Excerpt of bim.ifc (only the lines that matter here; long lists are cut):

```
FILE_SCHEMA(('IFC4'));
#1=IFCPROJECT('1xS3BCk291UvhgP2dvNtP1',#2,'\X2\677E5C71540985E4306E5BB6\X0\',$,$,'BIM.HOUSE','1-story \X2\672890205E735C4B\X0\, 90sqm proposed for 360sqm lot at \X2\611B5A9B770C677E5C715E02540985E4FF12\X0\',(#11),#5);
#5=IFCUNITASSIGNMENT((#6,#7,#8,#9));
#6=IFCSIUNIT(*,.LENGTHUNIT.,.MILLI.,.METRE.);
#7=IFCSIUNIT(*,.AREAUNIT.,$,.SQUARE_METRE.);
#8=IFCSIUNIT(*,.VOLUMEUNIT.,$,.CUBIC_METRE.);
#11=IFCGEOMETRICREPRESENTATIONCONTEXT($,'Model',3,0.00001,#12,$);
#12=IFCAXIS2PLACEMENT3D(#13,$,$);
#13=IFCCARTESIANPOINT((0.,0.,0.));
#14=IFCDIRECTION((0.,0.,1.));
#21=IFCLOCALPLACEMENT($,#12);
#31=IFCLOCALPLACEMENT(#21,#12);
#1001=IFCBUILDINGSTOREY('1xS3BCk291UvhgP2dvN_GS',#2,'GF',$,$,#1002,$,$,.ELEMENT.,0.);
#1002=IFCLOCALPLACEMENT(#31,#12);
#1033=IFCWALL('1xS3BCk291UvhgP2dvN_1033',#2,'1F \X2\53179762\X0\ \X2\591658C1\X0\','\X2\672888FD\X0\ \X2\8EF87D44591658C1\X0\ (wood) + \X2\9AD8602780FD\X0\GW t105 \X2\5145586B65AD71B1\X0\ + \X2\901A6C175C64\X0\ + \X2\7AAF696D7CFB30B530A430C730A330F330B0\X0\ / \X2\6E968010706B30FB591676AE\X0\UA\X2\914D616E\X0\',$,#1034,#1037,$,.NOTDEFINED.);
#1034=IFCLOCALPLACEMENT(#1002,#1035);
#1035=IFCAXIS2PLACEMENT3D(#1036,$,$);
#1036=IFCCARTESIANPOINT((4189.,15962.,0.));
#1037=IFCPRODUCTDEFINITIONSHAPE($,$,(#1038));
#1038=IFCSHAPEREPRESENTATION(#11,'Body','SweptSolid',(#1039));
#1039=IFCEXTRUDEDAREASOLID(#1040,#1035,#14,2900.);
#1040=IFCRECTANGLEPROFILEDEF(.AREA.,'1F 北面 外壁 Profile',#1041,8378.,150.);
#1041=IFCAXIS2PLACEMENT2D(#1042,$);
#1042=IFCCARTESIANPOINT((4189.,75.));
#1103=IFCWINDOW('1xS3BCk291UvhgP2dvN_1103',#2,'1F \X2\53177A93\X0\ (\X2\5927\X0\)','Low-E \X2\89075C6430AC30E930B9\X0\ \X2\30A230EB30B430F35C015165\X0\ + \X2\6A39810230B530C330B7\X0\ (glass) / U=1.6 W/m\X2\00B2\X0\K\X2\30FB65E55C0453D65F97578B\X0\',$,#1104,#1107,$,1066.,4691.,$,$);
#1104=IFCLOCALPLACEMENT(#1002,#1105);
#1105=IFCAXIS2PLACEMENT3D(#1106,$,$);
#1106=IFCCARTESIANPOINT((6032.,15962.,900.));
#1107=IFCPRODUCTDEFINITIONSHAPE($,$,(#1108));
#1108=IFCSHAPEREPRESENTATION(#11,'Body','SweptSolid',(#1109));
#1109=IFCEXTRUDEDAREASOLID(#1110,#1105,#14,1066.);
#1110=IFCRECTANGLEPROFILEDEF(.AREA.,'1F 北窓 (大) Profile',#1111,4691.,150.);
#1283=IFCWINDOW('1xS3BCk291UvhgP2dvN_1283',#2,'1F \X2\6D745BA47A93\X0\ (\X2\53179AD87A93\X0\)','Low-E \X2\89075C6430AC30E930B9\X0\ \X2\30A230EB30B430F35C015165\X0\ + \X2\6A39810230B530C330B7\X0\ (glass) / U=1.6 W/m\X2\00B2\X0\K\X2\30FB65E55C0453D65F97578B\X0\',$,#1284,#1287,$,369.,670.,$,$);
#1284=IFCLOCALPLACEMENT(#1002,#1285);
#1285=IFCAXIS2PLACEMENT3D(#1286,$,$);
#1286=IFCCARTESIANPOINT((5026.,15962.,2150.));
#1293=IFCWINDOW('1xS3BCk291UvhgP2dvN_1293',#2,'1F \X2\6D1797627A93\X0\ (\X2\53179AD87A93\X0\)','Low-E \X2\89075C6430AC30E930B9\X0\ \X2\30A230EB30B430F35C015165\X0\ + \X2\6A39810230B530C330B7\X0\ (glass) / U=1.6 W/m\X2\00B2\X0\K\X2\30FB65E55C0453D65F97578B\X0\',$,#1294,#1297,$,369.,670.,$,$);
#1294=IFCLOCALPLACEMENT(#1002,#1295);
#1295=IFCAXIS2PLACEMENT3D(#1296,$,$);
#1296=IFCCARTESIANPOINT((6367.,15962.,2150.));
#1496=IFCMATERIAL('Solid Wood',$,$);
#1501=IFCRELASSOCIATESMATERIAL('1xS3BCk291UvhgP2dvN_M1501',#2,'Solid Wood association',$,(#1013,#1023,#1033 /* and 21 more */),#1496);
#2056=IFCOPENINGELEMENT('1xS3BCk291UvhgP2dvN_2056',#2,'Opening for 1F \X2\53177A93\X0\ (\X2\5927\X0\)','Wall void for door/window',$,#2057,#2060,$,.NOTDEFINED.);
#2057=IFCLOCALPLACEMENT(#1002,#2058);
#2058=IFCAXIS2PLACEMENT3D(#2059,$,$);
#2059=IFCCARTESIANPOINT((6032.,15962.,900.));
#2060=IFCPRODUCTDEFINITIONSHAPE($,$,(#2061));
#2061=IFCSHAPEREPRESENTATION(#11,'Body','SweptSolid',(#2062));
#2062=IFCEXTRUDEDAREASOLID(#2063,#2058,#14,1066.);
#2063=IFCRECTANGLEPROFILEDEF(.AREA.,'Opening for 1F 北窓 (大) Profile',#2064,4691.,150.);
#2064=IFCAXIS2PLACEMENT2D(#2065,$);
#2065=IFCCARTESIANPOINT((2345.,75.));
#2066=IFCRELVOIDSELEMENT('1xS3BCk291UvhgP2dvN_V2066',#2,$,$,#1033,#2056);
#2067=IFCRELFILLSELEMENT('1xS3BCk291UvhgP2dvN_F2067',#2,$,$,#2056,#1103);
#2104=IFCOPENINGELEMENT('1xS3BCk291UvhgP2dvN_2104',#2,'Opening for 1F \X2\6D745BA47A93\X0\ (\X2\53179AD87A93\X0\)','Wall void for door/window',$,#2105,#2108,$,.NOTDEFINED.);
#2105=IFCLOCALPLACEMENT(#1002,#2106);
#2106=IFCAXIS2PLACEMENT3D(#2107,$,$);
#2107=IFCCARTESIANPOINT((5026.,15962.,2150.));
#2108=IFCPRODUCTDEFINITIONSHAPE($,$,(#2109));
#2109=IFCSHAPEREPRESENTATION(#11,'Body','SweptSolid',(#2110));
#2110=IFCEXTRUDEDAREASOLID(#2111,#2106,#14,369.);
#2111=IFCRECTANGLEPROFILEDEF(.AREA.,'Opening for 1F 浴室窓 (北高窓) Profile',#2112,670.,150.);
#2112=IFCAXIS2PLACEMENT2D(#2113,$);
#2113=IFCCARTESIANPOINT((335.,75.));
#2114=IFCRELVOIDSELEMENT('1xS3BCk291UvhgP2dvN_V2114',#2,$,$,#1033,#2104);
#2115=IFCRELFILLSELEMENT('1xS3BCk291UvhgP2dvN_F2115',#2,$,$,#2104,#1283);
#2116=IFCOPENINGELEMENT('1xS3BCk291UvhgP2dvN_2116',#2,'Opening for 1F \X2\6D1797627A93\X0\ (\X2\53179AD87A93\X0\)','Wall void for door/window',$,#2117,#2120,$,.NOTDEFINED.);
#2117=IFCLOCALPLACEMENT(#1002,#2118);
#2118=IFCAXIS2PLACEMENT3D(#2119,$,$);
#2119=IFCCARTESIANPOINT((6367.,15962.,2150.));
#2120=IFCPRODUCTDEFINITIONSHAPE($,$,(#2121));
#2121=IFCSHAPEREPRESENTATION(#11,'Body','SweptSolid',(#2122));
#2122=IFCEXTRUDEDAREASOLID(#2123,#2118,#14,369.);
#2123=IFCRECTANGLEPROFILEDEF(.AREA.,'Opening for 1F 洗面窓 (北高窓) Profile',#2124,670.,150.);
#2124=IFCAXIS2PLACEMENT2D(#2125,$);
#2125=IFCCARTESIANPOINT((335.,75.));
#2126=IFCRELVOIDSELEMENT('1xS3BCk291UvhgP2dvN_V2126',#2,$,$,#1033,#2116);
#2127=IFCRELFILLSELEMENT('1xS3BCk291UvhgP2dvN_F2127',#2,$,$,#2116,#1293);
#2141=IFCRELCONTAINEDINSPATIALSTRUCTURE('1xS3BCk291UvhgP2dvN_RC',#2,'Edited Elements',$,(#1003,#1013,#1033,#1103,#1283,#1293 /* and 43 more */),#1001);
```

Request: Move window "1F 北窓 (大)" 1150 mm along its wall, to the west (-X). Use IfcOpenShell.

```python
import ifcopenshell
import ifcopenshell.api.geometry
import ifcopenshell.util.placement
import ifcopenshell.util.unit

model = ifcopenshell.open("bim.ifc")
unit_scale = ifcopenshell.util.unit.calculate_unit_scale(model)

window = model.by_id(1103)
opening = window.FillsVoids[0].RelatingOpeningElement
wall = opening.VoidsElements[0].RelatingBuildingElement

wall_matrix = ifcopenshell.util.placement.get_local_placement(wall.ObjectPlacement)
shift = wall_matrix[:3, 0] * -1.15 / unit_scale
before = ifcopenshell.util.placement.get_local_placement(window.ObjectPlacement)[:3, 3].copy()

# The window is not placed relative to its opening, so move both.
for product in (opening, window):
    matrix = ifcopenshell.util.placement.get_local_placement(product.ObjectPlacement)
    matrix[:3, 3] += shift
    ifcopenshell.api.geometry.edit_object_placement(model, product=product, matrix=matrix, is_si=False)

after = ifcopenshell.util.placement.get_local_placement(window.ObjectPlacement)[:3, 3]
print("window moved by", (after - before).round(3) + 0.0)

model.write("bim_edited.ifc")
```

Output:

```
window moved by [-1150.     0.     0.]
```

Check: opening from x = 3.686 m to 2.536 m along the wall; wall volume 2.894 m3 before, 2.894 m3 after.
